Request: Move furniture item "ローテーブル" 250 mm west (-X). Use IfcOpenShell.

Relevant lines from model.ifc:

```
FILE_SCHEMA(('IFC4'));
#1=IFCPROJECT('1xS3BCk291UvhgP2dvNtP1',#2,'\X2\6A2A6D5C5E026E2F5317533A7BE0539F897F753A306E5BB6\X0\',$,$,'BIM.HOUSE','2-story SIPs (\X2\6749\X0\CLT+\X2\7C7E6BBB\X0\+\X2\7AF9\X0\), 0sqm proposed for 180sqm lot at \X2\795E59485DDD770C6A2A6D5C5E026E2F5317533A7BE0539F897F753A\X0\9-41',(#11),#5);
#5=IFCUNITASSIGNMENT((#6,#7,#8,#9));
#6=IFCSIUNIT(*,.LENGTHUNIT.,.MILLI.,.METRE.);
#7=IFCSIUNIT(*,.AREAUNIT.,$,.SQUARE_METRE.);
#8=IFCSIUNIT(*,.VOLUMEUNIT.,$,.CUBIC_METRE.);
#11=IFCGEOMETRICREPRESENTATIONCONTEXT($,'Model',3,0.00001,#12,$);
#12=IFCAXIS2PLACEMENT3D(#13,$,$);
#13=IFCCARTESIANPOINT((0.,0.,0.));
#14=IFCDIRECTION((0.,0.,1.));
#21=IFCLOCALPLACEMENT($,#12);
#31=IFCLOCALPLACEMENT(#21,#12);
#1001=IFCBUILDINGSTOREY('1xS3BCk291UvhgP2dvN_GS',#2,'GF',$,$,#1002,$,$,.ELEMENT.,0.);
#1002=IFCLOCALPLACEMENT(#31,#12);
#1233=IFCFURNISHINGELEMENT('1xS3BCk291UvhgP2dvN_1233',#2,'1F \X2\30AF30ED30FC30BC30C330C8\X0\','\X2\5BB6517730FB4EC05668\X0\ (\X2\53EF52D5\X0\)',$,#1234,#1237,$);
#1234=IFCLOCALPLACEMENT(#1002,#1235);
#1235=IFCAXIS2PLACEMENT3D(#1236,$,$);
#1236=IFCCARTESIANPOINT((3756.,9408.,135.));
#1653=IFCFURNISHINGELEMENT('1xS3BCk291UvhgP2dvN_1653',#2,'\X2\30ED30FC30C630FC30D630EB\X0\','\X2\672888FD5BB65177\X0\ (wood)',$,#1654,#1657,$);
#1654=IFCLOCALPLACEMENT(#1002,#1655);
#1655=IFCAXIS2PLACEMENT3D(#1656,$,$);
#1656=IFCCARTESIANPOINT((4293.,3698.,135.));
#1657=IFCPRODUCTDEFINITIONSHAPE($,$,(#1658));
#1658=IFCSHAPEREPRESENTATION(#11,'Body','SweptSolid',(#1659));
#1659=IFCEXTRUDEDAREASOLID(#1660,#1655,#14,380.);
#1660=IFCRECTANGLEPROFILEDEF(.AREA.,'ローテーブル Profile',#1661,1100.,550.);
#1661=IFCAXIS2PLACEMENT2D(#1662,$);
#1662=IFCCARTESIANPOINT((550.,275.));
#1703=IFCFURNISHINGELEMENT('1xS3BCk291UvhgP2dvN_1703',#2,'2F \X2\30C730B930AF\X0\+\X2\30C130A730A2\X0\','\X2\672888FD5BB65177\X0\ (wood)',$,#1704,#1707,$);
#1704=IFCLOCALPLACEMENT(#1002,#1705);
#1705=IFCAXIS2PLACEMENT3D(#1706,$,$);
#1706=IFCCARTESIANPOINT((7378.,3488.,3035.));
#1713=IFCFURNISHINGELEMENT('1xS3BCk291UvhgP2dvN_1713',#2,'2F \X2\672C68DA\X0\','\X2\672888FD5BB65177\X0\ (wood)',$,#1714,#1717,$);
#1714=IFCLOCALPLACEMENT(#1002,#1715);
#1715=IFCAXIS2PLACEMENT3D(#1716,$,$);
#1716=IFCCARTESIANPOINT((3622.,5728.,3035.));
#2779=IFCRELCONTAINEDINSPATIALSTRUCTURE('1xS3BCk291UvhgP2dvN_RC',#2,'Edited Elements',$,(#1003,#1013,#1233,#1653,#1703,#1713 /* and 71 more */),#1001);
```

```python
import ifcopenshell
import ifcopenshell.api.geometry
import ifcopenshell.util.placement
import ifcopenshell.util.unit

model = ifcopenshell.open("model.ifc")
unit_scale = ifcopenshell.util.unit.calculate_unit_scale(model)

item = model.by_id(1653)
matrix = ifcopenshell.util.placement.get_local_placement(item.ObjectPlacement)
matrix[0, 3] -= 0.25 / unit_scale
ifcopenshell.api.geometry.edit_object_placement(model, product=item, matrix=matrix, is_si=False)

print(ifcopenshell.util.placement.get_local_placement(item.ObjectPlacement).round(3) + 0.0)

model.write("model_edited.ifc")
```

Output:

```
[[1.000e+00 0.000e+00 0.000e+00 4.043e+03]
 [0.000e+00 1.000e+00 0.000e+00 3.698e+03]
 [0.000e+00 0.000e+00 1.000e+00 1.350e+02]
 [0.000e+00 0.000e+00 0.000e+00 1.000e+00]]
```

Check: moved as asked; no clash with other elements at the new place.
